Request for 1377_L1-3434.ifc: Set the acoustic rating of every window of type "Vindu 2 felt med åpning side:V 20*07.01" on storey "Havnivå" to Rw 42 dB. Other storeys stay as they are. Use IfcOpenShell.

First a look at what the model holds.

```python
import ifcopenshell
import ifcopenshell.util.element

model = ifcopenshell.open("1377_L1-3434.ifc")
print(model.schema)
storey = next(s for s in model.by_type("IfcBuildingStorey") if s.Name == "Havnivå")
windows = [e for e in ifcopenshell.util.element.get_decomposition(storey) if e.is_a("IfcWindow")]
seen = {}
for e in windows:
    element_type = ifcopenshell.util.element.get_type(e)
    key = (element_type.Name if element_type != e and element_type else None, ifcopenshell.util.element.get_pset(e, "Pset_WindowCommon", "AcousticRating"))
    seen[key] = seen.get(key, 0) + 1
for (name, value), count in sorted(seen.items(), key=str):
    print(count, "x", name, "|", value)
```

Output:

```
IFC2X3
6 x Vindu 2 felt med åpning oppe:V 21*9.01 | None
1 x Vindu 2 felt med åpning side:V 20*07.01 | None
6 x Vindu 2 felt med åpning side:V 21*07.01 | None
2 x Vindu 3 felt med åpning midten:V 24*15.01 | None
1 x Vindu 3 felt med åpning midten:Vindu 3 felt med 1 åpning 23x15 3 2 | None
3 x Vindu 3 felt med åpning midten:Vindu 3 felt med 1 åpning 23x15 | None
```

```python
import ifcopenshell
import ifcopenshell.api.pset
import ifcopenshell.util.element

model = ifcopenshell.open("1377_L1-3434.ifc")

storey = next(s for s in model.by_type("IfcBuildingStorey") if s.Name == "Havnivå")
windows = [e for e in ifcopenshell.util.element.get_decomposition(storey) if e.is_a("IfcWindow")]

count = 0
for e in windows:
    element_type = ifcopenshell.util.element.get_type(e)
    if element_type in (None, e) or element_type.Name != "Vindu 2 felt med åpning side:V 20*07.01":
        continue
    # add_pset returns the element's existing set when there is one.
    pset = ifcopenshell.api.pset.add_pset(model, product=e, name="Pset_WindowCommon")
    ifcopenshell.api.pset.edit_pset(model, pset=pset, properties={"AcousticRating": "Rw 42 dB"})
    count += 1

print(count, "windows updated")

model.write("1377_L1-3434_v2.ifc")
```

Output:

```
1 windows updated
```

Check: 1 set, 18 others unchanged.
